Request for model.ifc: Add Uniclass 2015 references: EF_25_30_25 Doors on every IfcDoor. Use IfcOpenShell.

First a look at what the model holds.

```python
import ifcopenshell

model = ifcopenshell.open("model.ifc")
print(model.schema)
print("classifications:", [c.Name for c in model.by_type("IfcClassification")])
for ifc_class in ("IfcDoor", "IfcRoof", "IfcStair", "IfcWall", "IfcWindow"):
    print(ifc_class, len(model.by_type(ifc_class)))
```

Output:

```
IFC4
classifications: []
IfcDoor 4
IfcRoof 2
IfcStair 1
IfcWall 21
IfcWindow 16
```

```python
import ifcopenshell
import ifcopenshell.api.classification

model = ifcopenshell.open("model.ifc")

system = ifcopenshell.api.classification.add_classification(model, classification="Uniclass 2015")

codes = {
    "IfcDoor": ("EF_25_30_25", "Doors"),
}
for ifc_class, (code, name) in codes.items():
    products = model.by_type(ifc_class)
    ifcopenshell.api.classification.add_reference(
        model, products=products, classification=system, identification=code, name=name
    )
    print(code, len(products))

model.write("model_edited.ifc")
```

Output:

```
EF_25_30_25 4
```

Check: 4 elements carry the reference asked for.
